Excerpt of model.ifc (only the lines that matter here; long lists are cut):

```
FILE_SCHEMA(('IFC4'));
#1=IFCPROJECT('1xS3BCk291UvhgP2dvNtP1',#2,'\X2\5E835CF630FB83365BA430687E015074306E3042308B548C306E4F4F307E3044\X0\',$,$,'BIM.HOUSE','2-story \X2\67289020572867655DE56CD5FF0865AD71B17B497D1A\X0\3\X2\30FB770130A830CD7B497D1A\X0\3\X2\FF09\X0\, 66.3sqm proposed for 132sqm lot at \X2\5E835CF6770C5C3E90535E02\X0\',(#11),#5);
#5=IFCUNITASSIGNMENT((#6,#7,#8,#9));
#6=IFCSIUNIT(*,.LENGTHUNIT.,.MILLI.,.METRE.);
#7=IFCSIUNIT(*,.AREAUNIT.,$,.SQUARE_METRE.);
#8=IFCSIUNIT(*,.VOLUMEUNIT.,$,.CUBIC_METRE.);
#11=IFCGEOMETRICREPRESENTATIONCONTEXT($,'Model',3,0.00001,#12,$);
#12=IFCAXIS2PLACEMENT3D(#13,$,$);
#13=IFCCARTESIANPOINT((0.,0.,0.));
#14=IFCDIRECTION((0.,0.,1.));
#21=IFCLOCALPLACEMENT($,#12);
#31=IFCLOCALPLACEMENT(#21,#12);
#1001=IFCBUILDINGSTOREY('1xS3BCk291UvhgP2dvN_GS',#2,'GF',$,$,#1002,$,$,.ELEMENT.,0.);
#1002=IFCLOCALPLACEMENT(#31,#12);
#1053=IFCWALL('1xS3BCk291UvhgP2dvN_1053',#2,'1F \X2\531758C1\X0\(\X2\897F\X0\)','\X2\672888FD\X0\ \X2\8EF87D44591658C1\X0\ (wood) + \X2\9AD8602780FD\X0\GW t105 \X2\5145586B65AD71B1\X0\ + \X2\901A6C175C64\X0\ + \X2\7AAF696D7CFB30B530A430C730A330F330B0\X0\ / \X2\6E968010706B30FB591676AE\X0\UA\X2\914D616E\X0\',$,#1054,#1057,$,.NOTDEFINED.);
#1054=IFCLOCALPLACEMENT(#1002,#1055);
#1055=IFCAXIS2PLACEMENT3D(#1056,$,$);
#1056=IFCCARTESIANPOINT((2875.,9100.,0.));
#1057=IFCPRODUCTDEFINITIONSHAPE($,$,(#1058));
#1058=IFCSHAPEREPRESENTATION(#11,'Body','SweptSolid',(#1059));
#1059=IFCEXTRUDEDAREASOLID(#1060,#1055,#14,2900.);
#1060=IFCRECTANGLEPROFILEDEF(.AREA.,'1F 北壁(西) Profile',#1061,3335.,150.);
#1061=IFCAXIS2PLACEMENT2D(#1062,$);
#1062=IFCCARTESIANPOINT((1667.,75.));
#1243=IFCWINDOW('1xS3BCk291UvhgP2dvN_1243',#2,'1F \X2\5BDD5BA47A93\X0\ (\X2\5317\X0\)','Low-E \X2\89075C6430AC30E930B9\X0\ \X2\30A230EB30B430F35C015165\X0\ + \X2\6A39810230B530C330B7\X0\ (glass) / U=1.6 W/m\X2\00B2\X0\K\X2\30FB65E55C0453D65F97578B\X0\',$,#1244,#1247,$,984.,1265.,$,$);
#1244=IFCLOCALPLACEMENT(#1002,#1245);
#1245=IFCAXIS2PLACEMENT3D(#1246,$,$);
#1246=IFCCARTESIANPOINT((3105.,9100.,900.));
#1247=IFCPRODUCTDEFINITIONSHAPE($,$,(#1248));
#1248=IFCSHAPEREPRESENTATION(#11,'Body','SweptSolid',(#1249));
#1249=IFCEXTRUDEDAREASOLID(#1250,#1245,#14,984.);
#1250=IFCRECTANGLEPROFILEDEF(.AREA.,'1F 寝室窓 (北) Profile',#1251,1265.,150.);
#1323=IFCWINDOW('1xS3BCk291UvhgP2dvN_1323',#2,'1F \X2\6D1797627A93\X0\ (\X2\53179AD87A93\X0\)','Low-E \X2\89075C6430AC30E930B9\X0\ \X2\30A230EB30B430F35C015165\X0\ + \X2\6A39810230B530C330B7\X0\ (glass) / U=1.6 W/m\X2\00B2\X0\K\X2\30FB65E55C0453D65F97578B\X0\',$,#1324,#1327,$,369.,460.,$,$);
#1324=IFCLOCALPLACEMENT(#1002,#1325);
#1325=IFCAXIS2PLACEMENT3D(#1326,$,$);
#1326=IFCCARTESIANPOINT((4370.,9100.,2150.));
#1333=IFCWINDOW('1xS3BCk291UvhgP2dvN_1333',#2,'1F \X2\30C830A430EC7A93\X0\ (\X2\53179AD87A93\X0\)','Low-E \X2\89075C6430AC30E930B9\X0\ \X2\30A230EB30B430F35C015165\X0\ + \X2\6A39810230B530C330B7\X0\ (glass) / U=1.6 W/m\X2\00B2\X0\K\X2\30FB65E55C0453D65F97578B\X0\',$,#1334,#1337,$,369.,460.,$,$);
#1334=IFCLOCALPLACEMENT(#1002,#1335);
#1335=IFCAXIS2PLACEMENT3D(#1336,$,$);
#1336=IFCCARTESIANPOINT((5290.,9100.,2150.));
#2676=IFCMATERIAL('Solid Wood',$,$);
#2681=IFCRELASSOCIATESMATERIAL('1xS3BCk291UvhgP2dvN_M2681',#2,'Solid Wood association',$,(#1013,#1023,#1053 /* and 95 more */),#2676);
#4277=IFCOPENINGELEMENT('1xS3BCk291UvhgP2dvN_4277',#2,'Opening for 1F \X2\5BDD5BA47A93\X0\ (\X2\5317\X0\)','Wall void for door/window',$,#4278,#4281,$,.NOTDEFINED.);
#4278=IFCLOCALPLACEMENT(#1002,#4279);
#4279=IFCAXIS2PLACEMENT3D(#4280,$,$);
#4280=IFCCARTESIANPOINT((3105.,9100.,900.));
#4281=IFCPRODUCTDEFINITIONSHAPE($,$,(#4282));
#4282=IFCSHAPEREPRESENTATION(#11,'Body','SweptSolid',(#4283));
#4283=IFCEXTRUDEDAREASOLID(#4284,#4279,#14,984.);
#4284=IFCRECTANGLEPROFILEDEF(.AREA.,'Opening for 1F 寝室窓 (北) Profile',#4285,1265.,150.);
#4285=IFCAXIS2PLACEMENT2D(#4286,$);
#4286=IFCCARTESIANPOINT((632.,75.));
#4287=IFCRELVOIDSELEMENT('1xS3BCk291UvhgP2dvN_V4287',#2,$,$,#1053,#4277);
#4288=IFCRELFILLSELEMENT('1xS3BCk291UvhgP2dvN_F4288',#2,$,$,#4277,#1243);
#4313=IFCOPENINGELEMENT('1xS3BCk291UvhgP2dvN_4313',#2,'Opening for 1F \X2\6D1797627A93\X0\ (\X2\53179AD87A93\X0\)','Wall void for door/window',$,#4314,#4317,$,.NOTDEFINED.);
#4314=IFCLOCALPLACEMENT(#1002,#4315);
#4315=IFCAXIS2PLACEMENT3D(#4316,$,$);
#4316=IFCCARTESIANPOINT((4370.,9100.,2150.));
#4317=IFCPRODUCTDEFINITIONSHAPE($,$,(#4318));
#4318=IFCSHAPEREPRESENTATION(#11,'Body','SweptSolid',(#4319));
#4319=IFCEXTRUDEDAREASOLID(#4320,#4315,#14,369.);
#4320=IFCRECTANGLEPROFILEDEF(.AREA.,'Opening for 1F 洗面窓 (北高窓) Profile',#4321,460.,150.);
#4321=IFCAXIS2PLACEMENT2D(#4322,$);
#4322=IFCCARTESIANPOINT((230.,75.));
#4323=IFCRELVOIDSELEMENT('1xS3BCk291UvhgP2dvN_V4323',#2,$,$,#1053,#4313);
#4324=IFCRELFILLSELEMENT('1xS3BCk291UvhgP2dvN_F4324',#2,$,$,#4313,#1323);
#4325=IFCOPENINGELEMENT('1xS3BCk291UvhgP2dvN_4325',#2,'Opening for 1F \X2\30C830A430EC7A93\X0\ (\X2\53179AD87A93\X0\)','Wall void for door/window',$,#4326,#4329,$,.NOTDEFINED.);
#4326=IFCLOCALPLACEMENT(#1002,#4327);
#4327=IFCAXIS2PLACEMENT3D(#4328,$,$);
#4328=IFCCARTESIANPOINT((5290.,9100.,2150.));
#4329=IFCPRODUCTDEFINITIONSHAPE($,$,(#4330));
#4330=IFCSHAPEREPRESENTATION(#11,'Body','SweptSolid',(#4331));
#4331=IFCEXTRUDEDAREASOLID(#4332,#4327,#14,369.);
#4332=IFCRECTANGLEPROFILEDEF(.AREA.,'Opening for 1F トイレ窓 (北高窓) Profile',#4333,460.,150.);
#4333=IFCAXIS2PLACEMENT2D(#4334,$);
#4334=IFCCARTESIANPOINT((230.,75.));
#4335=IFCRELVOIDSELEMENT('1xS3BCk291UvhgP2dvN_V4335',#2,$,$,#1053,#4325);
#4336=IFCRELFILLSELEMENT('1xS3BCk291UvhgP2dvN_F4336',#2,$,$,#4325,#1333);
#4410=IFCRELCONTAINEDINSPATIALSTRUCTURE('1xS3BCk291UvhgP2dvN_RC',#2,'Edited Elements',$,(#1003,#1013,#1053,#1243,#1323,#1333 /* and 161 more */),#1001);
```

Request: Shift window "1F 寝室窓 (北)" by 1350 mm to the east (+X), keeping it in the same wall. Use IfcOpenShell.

```python
import ifcopenshell
import ifcopenshell.api.geometry
import ifcopenshell.util.placement
import ifcopenshell.util.unit

model = ifcopenshell.open("model.ifc")
unit_scale = ifcopenshell.util.unit.calculate_unit_scale(model)

window = model.by_guid("1xS3BCk291UvhgP2dvN_1243")
opening = window.FillsVoids[0].RelatingOpeningElement
wall = opening.VoidsElements[0].RelatingBuildingElement

wall_matrix = ifcopenshell.util.placement.get_local_placement(wall.ObjectPlacement)
shift = wall_matrix[:3, 0] * 1.35 / unit_scale
before = ifcopenshell.util.placement.get_local_placement(window.ObjectPlacement)[:3, 3].copy()

# The window is not placed relative to its opening, so move both.
for product in (opening, window):
    matrix = ifcopenshell.util.placement.get_local_placement(product.ObjectPlacement)
    matrix[:3, 3] += shift
    ifcopenshell.api.geometry.edit_object_placement(model, product=product, matrix=matrix, is_si=False)

after = ifcopenshell.util.placement.get_local_placement(window.ObjectPlacement)[:3, 3]
print("window moved by", (after - before).round(3) + 0.0)

model.write("model-out.ifc")
```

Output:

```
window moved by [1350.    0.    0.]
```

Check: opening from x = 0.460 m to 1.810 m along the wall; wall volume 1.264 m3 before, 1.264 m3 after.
